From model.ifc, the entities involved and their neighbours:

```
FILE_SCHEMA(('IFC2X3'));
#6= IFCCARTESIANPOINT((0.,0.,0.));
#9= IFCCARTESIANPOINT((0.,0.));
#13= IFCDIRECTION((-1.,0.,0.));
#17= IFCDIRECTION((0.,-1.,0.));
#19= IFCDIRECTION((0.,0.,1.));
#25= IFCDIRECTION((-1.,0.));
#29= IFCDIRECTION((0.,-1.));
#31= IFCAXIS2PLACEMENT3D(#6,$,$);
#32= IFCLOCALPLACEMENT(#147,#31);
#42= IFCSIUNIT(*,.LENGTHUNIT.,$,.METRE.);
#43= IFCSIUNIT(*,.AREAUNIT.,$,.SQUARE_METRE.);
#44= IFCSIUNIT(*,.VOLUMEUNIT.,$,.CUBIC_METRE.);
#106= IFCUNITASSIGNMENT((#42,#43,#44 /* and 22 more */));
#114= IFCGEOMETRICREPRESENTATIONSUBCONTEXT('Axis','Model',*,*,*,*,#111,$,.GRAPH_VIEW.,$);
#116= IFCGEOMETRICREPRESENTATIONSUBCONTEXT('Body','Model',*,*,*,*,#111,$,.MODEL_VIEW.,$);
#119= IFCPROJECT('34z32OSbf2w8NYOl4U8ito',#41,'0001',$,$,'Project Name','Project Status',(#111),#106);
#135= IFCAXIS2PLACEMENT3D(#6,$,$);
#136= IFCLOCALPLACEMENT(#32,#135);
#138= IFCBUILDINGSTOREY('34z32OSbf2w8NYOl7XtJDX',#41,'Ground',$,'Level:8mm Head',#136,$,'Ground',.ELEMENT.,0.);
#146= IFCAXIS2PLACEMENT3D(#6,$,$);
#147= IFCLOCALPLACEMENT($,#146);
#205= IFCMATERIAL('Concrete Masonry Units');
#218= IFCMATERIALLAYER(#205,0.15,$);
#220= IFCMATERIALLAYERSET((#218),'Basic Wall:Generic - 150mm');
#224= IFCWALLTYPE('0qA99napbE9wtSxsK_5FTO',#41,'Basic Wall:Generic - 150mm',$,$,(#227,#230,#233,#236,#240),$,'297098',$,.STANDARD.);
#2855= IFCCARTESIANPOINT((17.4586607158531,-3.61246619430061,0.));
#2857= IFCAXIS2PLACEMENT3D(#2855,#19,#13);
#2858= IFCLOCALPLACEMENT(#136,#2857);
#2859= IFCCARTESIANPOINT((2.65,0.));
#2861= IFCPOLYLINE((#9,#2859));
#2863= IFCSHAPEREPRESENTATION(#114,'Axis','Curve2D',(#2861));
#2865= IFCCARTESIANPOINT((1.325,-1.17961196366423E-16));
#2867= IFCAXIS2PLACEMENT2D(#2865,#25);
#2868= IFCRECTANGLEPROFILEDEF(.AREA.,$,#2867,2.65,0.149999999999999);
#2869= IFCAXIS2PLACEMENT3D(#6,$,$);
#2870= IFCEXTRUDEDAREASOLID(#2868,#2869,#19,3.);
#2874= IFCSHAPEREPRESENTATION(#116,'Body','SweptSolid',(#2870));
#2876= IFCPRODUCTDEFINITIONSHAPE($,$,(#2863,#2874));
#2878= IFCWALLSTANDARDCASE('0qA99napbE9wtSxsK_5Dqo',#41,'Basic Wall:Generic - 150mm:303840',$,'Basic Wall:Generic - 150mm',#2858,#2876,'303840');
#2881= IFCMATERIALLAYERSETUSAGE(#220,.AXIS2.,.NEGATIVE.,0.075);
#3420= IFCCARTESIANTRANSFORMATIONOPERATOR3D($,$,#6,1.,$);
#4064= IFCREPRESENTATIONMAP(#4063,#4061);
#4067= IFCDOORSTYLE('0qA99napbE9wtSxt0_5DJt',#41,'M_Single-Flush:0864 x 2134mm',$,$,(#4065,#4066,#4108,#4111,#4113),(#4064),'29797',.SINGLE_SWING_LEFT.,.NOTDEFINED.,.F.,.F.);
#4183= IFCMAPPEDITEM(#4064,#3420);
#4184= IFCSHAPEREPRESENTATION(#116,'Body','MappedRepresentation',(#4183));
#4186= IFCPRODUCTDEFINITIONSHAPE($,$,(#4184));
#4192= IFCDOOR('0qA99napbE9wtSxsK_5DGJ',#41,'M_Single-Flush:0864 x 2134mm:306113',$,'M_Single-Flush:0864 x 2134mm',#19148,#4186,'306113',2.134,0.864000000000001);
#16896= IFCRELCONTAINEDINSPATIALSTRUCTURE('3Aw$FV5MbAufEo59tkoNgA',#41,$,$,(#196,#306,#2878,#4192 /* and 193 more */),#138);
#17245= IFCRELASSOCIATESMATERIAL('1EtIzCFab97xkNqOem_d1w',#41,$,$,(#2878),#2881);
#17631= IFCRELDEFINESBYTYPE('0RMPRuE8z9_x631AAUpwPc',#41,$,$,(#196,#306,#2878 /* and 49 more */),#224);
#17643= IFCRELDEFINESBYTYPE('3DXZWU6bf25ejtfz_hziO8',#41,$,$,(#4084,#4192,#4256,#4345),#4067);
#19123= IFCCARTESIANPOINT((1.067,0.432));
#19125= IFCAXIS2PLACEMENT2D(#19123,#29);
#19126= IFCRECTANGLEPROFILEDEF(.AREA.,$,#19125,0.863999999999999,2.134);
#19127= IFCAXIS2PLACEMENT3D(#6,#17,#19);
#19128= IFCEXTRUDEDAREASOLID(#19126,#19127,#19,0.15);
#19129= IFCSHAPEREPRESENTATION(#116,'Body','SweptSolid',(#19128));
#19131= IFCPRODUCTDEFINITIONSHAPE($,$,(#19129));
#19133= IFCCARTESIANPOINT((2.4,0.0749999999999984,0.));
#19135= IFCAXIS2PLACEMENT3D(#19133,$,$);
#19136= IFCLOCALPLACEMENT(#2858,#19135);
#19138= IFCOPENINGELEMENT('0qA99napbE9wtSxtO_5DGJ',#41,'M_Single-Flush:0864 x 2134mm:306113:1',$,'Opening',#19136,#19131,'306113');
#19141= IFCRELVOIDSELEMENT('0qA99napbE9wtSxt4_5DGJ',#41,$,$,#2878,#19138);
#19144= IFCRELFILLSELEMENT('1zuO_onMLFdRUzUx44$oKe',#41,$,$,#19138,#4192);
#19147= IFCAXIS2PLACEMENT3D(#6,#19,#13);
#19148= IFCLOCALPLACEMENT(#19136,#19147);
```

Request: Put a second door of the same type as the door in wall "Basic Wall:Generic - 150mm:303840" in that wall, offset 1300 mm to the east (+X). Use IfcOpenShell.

```python
import ifcopenshell
import ifcopenshell.api.feature
import ifcopenshell.api.geometry
import ifcopenshell.api.root
import ifcopenshell.geom
import ifcopenshell.util.element
import ifcopenshell.util.placement
import ifcopenshell.util.shape
import ifcopenshell.util.unit

model = ifcopenshell.open("model.ifc")
unit_scale = ifcopenshell.util.unit.calculate_unit_scale(model)
settings = ifcopenshell.geom.settings()


def volume(element):
    """Net volume in cubic metres, openings subtracted."""
    shape = ifcopenshell.geom.create_shape(settings, element)
    return ifcopenshell.util.shape.get_volume(shape.geometry)


def reuse_history(source, copy):
    """copy_class also copies each property set's owner history, people and application; keep the originals."""
    for rel in copy.IsDefinedBy:
        if rel.is_a("IfcRelDefinesByProperties") and (history := rel.RelatingPropertyDefinition.OwnerHistory):
            rel.RelatingPropertyDefinition.OwnerHistory = source.OwnerHistory
            ifcopenshell.util.element.remove_deep2(model, history)


door = model.by_guid("0qA99napbE9wtSxsK_5DGJ")
opening = door.FillsVoids[0].RelatingOpeningElement
wall = opening.VoidsElements[0].RelatingBuildingElement
before = volume(wall)
shift = ifcopenshell.util.placement.get_local_placement(wall.ObjectPlacement)[:3, 0] * -1.3 / unit_scale

# copy_class copies the void relationship, type, container and properties, but no geometry.
new_opening = ifcopenshell.api.root.copy_class(model, product=opening)
new_opening.Representation = ifcopenshell.util.element.copy_deep(
    model, opening.Representation, exclude=["IfcGeometricRepresentationContext", "IfcRepresentationMap"]
)
new_opening.Name = "M_Single-Flush:0864 x 2134mm"
new_opening.Tag = None
new_door = ifcopenshell.api.root.copy_class(model, product=door)
new_door.Representation = ifcopenshell.util.element.copy_deep(
    model, door.Representation, exclude=["IfcGeometricRepresentationContext", "IfcRepresentationMap"]
)
new_door.Name = "M_Single-Flush:0864 x 2134mm"
new_door.Tag = None
reuse_history(door, new_door)
fills = ifcopenshell.api.feature.add_filling(model, opening=new_opening, element=new_door)
fills.OwnerHistory = new_door.OwnerHistory  # required in IFC2X3

for old, new in ((opening, new_opening), (door, new_door)):
    matrix = ifcopenshell.util.placement.get_local_placement(old.ObjectPlacement)
    matrix[:3, 3] += shift
    ifcopenshell.api.geometry.edit_object_placement(model, product=new, matrix=matrix, is_si=False)

after = volume(wall)

print(f"wall volume {before:.3f} -> {after:.3f} m3")

model.write("model_v2.ifc")
```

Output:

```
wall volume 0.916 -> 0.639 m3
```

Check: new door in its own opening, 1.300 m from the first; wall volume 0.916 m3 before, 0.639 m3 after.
